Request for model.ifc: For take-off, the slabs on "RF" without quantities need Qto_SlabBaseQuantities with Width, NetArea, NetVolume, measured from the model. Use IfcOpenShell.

First a look at what the model holds.

```python
import ifcopenshell
import ifcopenshell.util.element
import ifcopenshell.util.unit

model = ifcopenshell.open("model.ifc")
print(model.schema)
for unit_type in ("LENGTHUNIT", "AREAUNIT", "VOLUMEUNIT"):
    print(unit_type, ifcopenshell.util.unit.calculate_unit_scale(model, unit_type))
storey = next(s for s in model.by_type("IfcBuildingStorey") if s.Name == "RF")
slabs = [e for e in ifcopenshell.util.element.get_decomposition(storey) if e.is_a("IfcSlab")]
for e in sorted(slabs, key=lambda e: e.id()):
    print(e.id(), e.is_a(), e.Name, list(ifcopenshell.util.element.get_psets(e, qtos_only=True)), sep=" | ")
```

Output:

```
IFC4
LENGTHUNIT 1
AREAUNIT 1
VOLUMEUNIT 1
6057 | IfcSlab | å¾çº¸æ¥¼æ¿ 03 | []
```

```python
import ifcopenshell
import ifcopenshell.api.pset
import ifcopenshell.geom
import ifcopenshell.util.element
import ifcopenshell.util.shape
import ifcopenshell.util.unit

model = ifcopenshell.open("model.ifc")
unit_scale = ifcopenshell.util.unit.calculate_unit_scale(model)
area_scale = ifcopenshell.util.unit.calculate_unit_scale(model, "AREAUNIT")
volume_scale = ifcopenshell.util.unit.calculate_unit_scale(model, "VOLUMEUNIT")
settings = ifcopenshell.geom.settings()

storey = next(s for s in model.by_type("IfcBuildingStorey") if s.Name == "RF")
slabs = [e for e in ifcopenshell.util.element.get_decomposition(storey) if e.is_a("IfcSlab")]

for e in sorted(slabs, key=lambda e: e.id()):
    if ifcopenshell.util.element.get_psets(e, qtos_only=True, should_inherit=False):
        continue
    # Geometry comes back in metres, in the element's own axes.
    shape = ifcopenshell.geom.create_shape(settings, e)
    values = {
        "Width": ifcopenshell.util.shape.get_z(shape.geometry) / unit_scale,
        "NetArea": ifcopenshell.util.shape.get_footprint_area(shape.geometry) / area_scale,
        "NetVolume": ifcopenshell.util.shape.get_volume(shape.geometry) / volume_scale,
    }
    qto = ifcopenshell.api.pset.add_qto(model, product=e, name="Qto_SlabBaseQuantities")
    ifcopenshell.api.pset.edit_qto(model, qto=qto, properties=values)
    print(e.id(), {k: round(v, 3) for k, v in values.items()})

model.write("model_edited.ifc")
```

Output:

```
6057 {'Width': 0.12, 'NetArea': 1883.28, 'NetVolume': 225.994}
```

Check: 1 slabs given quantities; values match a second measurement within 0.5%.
